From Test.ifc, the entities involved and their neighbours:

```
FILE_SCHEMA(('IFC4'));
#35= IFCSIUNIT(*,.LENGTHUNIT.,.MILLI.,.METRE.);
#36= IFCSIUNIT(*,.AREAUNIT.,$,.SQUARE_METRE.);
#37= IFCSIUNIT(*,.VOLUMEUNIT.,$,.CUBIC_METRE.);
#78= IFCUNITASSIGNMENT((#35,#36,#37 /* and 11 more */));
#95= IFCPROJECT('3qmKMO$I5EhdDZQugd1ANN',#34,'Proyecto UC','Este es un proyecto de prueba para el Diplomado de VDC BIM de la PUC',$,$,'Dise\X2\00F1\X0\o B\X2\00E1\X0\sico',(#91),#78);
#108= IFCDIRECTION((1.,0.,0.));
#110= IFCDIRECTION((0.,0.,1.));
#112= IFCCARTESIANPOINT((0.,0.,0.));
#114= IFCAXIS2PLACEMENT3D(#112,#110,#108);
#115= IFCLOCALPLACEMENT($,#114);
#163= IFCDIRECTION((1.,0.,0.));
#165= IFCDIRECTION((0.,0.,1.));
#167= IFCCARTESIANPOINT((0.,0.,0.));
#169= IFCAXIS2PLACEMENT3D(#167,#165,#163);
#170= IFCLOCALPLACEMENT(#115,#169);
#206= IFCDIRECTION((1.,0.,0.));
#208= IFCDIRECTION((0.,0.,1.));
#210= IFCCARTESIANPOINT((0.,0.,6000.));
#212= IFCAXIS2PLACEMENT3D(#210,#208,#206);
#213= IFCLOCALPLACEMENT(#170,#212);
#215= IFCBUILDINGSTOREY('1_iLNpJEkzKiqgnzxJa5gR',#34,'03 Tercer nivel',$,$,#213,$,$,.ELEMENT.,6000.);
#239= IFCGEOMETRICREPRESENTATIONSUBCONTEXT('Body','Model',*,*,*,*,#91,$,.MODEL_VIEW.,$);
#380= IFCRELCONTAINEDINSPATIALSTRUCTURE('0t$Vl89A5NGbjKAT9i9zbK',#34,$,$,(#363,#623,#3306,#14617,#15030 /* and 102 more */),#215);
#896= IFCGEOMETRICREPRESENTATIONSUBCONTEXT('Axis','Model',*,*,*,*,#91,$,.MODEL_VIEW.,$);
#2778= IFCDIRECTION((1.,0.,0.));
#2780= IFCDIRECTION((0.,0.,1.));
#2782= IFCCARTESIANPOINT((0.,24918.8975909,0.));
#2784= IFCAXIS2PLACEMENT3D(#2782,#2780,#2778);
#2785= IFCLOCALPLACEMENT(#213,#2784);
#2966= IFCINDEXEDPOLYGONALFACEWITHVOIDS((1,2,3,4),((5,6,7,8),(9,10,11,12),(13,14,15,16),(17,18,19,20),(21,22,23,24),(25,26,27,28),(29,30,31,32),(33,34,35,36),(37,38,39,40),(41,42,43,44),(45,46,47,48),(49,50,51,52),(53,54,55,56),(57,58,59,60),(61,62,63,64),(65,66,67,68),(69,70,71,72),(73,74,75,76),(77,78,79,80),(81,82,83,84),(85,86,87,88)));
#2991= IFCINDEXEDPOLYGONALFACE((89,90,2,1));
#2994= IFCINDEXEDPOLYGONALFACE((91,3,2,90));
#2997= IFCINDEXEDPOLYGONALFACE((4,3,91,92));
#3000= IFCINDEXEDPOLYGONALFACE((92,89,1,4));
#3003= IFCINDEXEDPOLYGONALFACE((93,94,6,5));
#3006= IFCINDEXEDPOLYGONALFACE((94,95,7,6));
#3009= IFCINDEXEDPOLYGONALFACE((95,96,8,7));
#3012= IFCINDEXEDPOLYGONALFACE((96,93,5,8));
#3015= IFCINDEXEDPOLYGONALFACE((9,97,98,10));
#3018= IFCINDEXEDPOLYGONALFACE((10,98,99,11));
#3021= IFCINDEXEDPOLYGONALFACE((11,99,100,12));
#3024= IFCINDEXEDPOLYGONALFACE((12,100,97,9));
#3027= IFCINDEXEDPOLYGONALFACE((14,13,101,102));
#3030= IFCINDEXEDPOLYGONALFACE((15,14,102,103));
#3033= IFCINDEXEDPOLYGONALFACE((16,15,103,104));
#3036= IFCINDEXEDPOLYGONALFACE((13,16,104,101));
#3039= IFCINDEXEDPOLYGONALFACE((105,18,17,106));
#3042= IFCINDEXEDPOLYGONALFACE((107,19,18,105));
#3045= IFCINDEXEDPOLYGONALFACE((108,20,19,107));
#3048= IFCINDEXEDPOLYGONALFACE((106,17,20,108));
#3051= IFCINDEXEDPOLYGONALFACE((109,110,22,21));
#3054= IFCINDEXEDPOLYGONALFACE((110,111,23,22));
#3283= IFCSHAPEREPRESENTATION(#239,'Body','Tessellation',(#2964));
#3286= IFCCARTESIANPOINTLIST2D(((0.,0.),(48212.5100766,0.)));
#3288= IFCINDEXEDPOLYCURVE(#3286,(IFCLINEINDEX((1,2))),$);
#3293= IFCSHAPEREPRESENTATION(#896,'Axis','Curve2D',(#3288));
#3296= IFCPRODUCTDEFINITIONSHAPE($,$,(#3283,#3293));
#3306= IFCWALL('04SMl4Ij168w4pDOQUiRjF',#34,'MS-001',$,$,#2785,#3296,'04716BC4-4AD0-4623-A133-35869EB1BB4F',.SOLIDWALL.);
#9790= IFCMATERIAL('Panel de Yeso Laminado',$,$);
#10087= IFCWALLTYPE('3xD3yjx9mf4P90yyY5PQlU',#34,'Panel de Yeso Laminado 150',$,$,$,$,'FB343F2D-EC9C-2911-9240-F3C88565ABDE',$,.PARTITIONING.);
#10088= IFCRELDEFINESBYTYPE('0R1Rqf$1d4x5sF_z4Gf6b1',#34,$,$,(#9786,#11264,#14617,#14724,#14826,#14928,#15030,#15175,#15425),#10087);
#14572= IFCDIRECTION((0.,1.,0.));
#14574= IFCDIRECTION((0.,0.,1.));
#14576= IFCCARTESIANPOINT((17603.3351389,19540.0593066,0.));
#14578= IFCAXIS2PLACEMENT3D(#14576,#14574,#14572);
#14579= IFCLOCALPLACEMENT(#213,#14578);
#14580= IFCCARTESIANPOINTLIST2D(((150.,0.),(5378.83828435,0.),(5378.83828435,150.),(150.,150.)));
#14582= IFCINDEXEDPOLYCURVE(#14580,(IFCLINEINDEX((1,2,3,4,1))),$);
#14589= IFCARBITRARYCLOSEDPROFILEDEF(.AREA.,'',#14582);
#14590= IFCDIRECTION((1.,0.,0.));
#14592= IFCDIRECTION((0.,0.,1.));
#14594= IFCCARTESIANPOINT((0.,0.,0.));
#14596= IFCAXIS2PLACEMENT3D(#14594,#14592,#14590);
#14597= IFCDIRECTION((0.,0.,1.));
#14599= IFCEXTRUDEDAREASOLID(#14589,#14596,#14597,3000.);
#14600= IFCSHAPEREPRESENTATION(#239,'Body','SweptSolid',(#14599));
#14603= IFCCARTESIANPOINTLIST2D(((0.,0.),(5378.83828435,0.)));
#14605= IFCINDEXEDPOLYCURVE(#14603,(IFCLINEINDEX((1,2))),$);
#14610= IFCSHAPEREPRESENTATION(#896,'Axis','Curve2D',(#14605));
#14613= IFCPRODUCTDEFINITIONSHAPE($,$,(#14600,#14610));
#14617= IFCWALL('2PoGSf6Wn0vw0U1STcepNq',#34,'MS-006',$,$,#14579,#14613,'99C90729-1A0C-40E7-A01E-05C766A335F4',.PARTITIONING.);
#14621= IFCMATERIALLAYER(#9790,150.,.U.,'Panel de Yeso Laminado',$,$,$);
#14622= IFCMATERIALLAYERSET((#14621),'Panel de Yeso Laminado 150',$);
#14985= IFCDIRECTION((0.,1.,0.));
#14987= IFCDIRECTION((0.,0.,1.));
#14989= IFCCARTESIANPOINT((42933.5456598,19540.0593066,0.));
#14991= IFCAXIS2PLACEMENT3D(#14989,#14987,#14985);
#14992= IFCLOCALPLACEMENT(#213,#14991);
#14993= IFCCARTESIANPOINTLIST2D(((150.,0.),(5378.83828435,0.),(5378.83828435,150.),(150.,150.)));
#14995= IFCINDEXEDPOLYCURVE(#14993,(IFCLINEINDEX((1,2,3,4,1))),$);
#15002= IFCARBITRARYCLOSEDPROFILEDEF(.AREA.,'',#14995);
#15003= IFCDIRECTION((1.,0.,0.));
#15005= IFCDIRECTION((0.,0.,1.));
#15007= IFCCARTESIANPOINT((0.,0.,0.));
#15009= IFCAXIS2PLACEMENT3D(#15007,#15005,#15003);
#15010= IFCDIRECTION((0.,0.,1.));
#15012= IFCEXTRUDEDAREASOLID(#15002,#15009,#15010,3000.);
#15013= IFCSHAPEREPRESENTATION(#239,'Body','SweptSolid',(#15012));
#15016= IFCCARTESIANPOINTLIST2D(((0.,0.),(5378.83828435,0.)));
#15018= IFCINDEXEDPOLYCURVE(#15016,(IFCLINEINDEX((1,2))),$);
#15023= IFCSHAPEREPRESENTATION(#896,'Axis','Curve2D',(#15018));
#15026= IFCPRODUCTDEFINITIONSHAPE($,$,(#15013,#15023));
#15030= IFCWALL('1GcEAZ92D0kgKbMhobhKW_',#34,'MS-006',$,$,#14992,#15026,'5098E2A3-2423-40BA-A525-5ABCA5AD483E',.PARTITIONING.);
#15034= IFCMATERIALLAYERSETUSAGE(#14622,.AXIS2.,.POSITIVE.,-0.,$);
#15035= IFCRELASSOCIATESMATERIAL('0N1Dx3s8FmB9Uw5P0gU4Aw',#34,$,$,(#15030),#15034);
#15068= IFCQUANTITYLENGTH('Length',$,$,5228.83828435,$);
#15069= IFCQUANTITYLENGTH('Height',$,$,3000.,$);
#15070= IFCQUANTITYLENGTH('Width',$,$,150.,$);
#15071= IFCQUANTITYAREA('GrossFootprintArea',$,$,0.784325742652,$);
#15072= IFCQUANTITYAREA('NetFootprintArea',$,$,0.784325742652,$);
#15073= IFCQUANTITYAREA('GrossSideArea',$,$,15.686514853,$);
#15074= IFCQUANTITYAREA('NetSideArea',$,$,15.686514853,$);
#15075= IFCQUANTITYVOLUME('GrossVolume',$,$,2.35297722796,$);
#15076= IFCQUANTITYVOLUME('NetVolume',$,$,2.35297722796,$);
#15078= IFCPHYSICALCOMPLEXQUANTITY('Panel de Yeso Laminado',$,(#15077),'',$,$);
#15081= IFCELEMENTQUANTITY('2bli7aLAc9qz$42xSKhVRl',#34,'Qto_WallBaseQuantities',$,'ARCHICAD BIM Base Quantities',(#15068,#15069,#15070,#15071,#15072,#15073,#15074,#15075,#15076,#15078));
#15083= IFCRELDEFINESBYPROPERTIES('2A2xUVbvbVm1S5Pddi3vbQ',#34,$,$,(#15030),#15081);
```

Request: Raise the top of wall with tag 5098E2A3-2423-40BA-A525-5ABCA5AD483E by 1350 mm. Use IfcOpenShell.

```python
import ifcopenshell
import ifcopenshell.api.pset
import ifcopenshell.geom
import ifcopenshell.util.element
import ifcopenshell.util.representation
import ifcopenshell.util.shape
import ifcopenshell.util.unit

model = ifcopenshell.open("Test.ifc")
unit_scale = ifcopenshell.util.unit.calculate_unit_scale(model)
area_scale = ifcopenshell.util.unit.calculate_unit_scale(model, "AREAUNIT")
volume_scale = ifcopenshell.util.unit.calculate_unit_scale(model, "VOLUMEUNIT")
settings = ifcopenshell.geom.settings()


def volume(element):
    """Net volume in cubic metres, openings subtracted."""
    shape = ifcopenshell.geom.create_shape(settings, element)
    return ifcopenshell.util.shape.get_volume(shape.geometry)


wall = model.by_id(15030)
before = volume(wall)

body = ifcopenshell.util.representation.get_representation(wall, "Model", "Body")
solid = body.Items[0]
old_height = solid.Depth
solid.Depth += 1350.0
after = volume(wall)
thickness = 0.15  # wall thickness in metres

# Update the stored height, areas and volumes.
qto = model.by_id(ifcopenshell.util.element.get_pset(wall, "Qto_WallBaseQuantities", should_inherit=False)["id"])
ifcopenshell.api.pset.edit_qto(model, qto=qto, properties={
    "Height": solid.Depth,
    "GrossSideArea": ifcopenshell.util.element.get_pset(wall, "Qto_WallBaseQuantities", "GrossSideArea") * solid.Depth / old_height,
    "NetSideArea": after / thickness / area_scale,
    "GrossVolume": ifcopenshell.util.element.get_pset(wall, "Qto_WallBaseQuantities", "GrossVolume") * solid.Depth / old_height,
    "NetVolume": after / volume_scale,
})

print(f"height {old_height:g} -> {solid.Depth:g}, volume {before:.3f} -> {after:.3f} m3")

model.write("Test-out.ifc")
```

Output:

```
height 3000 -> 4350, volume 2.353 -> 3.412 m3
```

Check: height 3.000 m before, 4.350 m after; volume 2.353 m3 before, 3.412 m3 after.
